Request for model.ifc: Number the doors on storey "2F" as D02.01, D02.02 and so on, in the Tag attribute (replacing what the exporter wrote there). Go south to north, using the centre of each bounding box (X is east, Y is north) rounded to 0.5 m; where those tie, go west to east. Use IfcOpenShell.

First a look at what the model holds.

```python
import ifcopenshell
import ifcopenshell.util.element
import ifcopenshell.util.placement

model = ifcopenshell.open("model.ifc")
print(model.schema)
storey = next(s for s in model.by_type("IfcBuildingStorey") if s.Name == "2F")
doors = [e for e in ifcopenshell.util.element.get_decomposition(storey) if e.is_a("IfcDoor")]
for e in sorted(doors, key=lambda e: e.id()):
    origin = ifcopenshell.util.placement.get_local_placement(e.ObjectPlacement)[:3, 3]
    print(e.id(), e.Tag, e.Name, origin.round(2) + 0.0, sep=" | ")
```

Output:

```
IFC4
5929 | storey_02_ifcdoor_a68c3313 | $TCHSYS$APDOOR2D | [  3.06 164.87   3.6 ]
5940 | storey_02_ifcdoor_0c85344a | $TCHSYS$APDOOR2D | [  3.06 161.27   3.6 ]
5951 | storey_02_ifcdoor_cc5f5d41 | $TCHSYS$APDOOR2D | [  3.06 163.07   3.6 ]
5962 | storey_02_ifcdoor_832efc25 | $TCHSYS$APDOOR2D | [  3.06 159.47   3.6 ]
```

```python
import ifcopenshell
import ifcopenshell.geom
import ifcopenshell.util.element
import ifcopenshell.util.shape

model = ifcopenshell.open("model.ifc")
settings = ifcopenshell.geom.settings()
settings.set("use-world-coords", True)


def centre(element):
    shape = ifcopenshell.geom.create_shape(settings, element)
    return ifcopenshell.util.shape.get_bbox_centroid(shape.geometry)


storey = next(s for s in model.by_type("IfcBuildingStorey") if s.Name == "2F")
doors = [e for e in ifcopenshell.util.element.get_decomposition(storey) if e.is_a("IfcDoor")]

# Insertion points can sit at a corner or the storey origin, so sort by the geometry (in metres).
centres = {e: centre(e) for e in doors}
doors.sort(key=lambda e: (round(centres[e][1] / 0.5), centres[e][0]))

for i, e in enumerate(doors, start=1):
    number = f"D02.{i:02d}"
    e.Tag = number
    print(e.id(), number)

model.write("model_edited.ifc")
```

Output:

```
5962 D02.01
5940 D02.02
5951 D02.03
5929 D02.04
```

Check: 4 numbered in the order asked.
